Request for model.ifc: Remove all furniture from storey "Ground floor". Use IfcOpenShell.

First a look at what the model holds.

```python
import ifcopenshell
import ifcopenshell.util.element

model = ifcopenshell.open("model.ifc")
print(model.schema)
storey = next(s for s in model.by_type("IfcBuildingStorey") if s.Name == "Ground floor")
furniture = [e for e in ifcopenshell.util.element.get_decomposition(storey) if e.is_a("IfcFurnishingElement")]
seen = {}
for e in furniture:
    element_type = ifcopenshell.util.element.get_type(e)
    name = element_type.Name if element_type not in (None, e) else None
    seen[name] = seen.get(name, 0) + 1
for name, count in sorted(seen.items(), key=str):
    print(count, "x", name)
```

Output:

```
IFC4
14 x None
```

```python
import ifcopenshell
import ifcopenshell.api.root
import ifcopenshell.util.element

model = ifcopenshell.open("model.ifc")

storey = next(s for s in model.by_type("IfcBuildingStorey") if s.Name == "Ground floor")
furniture = [e for e in ifcopenshell.util.element.get_decomposition(storey) if e.is_a("IfcFurnishingElement")]

for e in furniture:
    ifcopenshell.api.root.remove_product(model, product=e)
print(len(furniture), "removed")

model.write("model_v2.ifc")
```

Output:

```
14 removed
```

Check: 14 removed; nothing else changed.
